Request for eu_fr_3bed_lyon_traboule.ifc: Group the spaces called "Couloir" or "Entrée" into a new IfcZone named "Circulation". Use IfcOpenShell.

First a look at what the model holds.

```python
import ifcopenshell

model = ifcopenshell.open("eu_fr_3bed_lyon_traboule.ifc")
print(model.schema)
seen = {}
for space in model.by_type("IfcSpace"):
    seen[space.LongName] = seen.get(space.LongName, 0) + 1
for name, count in sorted(seen.items(), key=str):
    print(count, "x", name)
print("zones:", [z.Name for z in model.by_type("IfcZone")][:20])
```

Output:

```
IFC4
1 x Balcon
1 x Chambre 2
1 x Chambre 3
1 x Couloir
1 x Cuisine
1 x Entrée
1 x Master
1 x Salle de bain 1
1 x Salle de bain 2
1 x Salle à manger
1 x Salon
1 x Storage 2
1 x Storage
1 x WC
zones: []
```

```python
import ifcopenshell
import ifcopenshell.api.group
import ifcopenshell.api.root

model = ifcopenshell.open("eu_fr_3bed_lyon_traboule.ifc")

names = {"Couloir", "Entrée"}
spaces = [s for s in model.by_type("IfcSpace") if s.LongName in names]

zone = ifcopenshell.api.root.create_entity(model, ifc_class="IfcZone", name="Circulation")
ifcopenshell.api.group.assign_group(model, products=spaces, group=zone)
print(len(spaces), "spaces in", zone.Name)

model.write("eu_fr_3bed_lyon_traboule_updated.ifc")
```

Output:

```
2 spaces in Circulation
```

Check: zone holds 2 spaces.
